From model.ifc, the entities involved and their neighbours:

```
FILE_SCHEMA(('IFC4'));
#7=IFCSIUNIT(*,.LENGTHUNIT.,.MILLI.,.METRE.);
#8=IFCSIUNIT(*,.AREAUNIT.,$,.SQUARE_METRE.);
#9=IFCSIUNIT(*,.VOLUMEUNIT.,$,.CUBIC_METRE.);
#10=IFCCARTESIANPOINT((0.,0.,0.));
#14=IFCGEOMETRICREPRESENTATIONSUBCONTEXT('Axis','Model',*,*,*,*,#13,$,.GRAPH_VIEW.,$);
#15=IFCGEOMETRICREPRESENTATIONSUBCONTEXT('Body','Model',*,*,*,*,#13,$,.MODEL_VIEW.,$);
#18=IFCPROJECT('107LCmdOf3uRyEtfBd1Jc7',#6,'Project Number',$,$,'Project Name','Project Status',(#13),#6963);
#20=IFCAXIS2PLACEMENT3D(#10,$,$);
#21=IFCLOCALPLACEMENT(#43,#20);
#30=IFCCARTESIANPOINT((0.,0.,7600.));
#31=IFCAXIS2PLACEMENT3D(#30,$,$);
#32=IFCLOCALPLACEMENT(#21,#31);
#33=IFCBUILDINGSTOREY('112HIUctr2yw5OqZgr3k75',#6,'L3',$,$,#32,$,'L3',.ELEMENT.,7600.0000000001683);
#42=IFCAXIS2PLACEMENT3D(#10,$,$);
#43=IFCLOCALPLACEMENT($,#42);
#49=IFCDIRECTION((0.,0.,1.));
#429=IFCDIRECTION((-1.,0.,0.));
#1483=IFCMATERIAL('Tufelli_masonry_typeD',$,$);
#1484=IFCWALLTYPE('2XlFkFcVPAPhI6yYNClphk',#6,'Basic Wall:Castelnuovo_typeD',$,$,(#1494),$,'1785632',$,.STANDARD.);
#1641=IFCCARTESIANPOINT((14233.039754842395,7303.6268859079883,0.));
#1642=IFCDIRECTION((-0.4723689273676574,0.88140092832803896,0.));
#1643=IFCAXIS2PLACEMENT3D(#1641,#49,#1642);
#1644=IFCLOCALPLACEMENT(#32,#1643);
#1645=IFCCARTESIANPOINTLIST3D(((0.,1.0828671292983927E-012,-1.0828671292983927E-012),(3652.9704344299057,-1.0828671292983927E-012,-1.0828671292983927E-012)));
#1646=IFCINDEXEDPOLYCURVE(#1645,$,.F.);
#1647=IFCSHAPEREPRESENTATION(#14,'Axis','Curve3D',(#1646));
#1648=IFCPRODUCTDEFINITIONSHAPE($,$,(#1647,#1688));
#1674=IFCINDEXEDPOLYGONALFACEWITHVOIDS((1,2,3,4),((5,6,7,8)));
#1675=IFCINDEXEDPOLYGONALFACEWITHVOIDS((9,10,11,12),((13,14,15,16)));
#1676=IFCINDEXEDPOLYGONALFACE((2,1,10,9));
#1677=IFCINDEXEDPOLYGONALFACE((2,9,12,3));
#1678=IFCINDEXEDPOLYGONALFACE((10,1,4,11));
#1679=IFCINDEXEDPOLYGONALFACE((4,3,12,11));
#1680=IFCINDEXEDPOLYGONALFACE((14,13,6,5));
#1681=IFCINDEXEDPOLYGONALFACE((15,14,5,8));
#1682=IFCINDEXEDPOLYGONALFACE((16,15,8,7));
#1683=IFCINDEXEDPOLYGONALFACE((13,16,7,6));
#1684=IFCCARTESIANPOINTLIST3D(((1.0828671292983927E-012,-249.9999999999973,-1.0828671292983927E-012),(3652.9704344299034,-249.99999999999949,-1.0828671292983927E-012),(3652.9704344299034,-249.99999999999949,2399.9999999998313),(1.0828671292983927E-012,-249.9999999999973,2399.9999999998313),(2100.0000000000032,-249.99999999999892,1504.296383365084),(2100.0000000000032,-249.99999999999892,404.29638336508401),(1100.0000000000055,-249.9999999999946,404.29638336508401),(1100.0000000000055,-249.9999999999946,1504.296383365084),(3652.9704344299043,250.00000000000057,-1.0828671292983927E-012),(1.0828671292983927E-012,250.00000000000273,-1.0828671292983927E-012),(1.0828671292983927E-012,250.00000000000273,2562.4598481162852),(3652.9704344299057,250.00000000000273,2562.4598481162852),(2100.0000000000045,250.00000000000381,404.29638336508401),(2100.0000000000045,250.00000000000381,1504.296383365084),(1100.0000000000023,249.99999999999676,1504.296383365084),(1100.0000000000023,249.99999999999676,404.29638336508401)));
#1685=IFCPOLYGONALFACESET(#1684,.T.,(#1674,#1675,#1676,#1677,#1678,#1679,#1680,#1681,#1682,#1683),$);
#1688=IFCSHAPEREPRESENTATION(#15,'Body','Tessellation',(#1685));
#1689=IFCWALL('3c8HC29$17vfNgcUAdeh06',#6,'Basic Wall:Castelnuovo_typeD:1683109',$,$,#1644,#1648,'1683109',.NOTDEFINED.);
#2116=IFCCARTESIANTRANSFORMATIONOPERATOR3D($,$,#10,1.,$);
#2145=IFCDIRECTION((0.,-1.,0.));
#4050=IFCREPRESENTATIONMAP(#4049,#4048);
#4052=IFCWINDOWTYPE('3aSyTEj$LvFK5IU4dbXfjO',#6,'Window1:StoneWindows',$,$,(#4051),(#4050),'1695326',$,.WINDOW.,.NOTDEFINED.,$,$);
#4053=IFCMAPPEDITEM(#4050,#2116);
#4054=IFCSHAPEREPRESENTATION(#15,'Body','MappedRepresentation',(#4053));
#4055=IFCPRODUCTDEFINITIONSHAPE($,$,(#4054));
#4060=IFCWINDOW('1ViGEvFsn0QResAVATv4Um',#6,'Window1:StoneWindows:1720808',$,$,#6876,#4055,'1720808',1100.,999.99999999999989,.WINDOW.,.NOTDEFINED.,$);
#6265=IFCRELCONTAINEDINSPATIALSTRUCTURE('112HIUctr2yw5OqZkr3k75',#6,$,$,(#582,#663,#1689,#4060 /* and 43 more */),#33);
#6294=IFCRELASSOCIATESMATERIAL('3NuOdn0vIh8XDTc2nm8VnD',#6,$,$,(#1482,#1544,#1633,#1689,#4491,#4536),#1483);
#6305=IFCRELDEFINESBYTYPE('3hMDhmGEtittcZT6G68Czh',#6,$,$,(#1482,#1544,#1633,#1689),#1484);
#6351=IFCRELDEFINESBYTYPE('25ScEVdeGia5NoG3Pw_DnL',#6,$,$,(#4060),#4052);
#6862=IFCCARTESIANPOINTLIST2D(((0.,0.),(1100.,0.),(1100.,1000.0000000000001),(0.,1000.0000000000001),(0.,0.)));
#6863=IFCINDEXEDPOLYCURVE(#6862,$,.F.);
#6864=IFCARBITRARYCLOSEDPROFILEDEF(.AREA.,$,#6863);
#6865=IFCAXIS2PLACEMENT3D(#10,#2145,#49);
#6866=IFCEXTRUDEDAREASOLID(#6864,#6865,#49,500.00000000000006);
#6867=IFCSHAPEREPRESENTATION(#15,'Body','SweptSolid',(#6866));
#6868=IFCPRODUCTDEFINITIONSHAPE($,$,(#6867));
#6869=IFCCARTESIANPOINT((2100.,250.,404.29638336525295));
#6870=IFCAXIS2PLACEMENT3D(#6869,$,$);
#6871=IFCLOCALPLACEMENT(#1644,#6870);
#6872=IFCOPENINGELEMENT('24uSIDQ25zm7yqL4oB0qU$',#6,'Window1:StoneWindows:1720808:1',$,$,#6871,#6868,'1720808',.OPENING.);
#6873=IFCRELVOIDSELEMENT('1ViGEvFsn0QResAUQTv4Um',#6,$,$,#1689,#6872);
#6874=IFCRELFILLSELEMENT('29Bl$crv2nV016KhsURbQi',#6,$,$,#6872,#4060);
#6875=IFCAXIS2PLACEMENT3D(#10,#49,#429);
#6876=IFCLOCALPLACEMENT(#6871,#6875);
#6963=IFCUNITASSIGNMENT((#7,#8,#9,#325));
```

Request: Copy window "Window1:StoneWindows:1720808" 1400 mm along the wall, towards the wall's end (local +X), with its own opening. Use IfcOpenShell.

```python
import ifcopenshell
import ifcopenshell.api.feature
import ifcopenshell.api.geometry
import ifcopenshell.api.root
import ifcopenshell.geom
import ifcopenshell.util.element
import ifcopenshell.util.placement
import ifcopenshell.util.shape
import ifcopenshell.util.unit

model = ifcopenshell.open("model.ifc")
unit_scale = ifcopenshell.util.unit.calculate_unit_scale(model)
settings = ifcopenshell.geom.settings()


def volume(element):
    """Net volume in cubic metres, openings subtracted."""
    shape = ifcopenshell.geom.create_shape(settings, element)
    return ifcopenshell.util.shape.get_volume(shape.geometry)


def reuse_history(source, copy):
    """copy_class also copies each property set's owner history, people and application; keep the originals."""
    for rel in copy.IsDefinedBy:
        if rel.is_a("IfcRelDefinesByProperties") and (history := rel.RelatingPropertyDefinition.OwnerHistory):
            rel.RelatingPropertyDefinition.OwnerHistory = source.OwnerHistory
            ifcopenshell.util.element.remove_deep2(model, history)


window = model.by_id(4060)
opening = window.FillsVoids[0].RelatingOpeningElement
wall = opening.VoidsElements[0].RelatingBuildingElement
before = volume(wall)
shift = ifcopenshell.util.placement.get_local_placement(wall.ObjectPlacement)[:3, 0] * 1.4 / unit_scale

# copy_class copies the void relationship, type, container and properties, but no geometry.
new_opening = ifcopenshell.api.root.copy_class(model, product=opening)
new_opening.Representation = ifcopenshell.util.element.copy_deep(
    model, opening.Representation, exclude=["IfcGeometricRepresentationContext", "IfcRepresentationMap"]
)
new_opening.Name = "Window1:StoneWindows"
new_opening.Tag = None
new_window = ifcopenshell.api.root.copy_class(model, product=window)
new_window.Representation = ifcopenshell.util.element.copy_deep(
    model, window.Representation, exclude=["IfcGeometricRepresentationContext", "IfcRepresentationMap"]
)
new_window.Name = "Window1:StoneWindows"
new_window.Tag = None
reuse_history(window, new_window)
ifcopenshell.api.feature.add_filling(model, opening=new_opening, element=new_window)

for old, new in ((opening, new_opening), (window, new_window)):
    matrix = ifcopenshell.util.placement.get_local_placement(old.ObjectPlacement)
    matrix[:3, 3] += shift
    ifcopenshell.api.geometry.edit_object_placement(model, product=new, matrix=matrix, is_si=False)

after = volume(wall)

print(f"wall volume {before:.3f} -> {after:.3f} m3")

model.write("model_v2.ifc")
```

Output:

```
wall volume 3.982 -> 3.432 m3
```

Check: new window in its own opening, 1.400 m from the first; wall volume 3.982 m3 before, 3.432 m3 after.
